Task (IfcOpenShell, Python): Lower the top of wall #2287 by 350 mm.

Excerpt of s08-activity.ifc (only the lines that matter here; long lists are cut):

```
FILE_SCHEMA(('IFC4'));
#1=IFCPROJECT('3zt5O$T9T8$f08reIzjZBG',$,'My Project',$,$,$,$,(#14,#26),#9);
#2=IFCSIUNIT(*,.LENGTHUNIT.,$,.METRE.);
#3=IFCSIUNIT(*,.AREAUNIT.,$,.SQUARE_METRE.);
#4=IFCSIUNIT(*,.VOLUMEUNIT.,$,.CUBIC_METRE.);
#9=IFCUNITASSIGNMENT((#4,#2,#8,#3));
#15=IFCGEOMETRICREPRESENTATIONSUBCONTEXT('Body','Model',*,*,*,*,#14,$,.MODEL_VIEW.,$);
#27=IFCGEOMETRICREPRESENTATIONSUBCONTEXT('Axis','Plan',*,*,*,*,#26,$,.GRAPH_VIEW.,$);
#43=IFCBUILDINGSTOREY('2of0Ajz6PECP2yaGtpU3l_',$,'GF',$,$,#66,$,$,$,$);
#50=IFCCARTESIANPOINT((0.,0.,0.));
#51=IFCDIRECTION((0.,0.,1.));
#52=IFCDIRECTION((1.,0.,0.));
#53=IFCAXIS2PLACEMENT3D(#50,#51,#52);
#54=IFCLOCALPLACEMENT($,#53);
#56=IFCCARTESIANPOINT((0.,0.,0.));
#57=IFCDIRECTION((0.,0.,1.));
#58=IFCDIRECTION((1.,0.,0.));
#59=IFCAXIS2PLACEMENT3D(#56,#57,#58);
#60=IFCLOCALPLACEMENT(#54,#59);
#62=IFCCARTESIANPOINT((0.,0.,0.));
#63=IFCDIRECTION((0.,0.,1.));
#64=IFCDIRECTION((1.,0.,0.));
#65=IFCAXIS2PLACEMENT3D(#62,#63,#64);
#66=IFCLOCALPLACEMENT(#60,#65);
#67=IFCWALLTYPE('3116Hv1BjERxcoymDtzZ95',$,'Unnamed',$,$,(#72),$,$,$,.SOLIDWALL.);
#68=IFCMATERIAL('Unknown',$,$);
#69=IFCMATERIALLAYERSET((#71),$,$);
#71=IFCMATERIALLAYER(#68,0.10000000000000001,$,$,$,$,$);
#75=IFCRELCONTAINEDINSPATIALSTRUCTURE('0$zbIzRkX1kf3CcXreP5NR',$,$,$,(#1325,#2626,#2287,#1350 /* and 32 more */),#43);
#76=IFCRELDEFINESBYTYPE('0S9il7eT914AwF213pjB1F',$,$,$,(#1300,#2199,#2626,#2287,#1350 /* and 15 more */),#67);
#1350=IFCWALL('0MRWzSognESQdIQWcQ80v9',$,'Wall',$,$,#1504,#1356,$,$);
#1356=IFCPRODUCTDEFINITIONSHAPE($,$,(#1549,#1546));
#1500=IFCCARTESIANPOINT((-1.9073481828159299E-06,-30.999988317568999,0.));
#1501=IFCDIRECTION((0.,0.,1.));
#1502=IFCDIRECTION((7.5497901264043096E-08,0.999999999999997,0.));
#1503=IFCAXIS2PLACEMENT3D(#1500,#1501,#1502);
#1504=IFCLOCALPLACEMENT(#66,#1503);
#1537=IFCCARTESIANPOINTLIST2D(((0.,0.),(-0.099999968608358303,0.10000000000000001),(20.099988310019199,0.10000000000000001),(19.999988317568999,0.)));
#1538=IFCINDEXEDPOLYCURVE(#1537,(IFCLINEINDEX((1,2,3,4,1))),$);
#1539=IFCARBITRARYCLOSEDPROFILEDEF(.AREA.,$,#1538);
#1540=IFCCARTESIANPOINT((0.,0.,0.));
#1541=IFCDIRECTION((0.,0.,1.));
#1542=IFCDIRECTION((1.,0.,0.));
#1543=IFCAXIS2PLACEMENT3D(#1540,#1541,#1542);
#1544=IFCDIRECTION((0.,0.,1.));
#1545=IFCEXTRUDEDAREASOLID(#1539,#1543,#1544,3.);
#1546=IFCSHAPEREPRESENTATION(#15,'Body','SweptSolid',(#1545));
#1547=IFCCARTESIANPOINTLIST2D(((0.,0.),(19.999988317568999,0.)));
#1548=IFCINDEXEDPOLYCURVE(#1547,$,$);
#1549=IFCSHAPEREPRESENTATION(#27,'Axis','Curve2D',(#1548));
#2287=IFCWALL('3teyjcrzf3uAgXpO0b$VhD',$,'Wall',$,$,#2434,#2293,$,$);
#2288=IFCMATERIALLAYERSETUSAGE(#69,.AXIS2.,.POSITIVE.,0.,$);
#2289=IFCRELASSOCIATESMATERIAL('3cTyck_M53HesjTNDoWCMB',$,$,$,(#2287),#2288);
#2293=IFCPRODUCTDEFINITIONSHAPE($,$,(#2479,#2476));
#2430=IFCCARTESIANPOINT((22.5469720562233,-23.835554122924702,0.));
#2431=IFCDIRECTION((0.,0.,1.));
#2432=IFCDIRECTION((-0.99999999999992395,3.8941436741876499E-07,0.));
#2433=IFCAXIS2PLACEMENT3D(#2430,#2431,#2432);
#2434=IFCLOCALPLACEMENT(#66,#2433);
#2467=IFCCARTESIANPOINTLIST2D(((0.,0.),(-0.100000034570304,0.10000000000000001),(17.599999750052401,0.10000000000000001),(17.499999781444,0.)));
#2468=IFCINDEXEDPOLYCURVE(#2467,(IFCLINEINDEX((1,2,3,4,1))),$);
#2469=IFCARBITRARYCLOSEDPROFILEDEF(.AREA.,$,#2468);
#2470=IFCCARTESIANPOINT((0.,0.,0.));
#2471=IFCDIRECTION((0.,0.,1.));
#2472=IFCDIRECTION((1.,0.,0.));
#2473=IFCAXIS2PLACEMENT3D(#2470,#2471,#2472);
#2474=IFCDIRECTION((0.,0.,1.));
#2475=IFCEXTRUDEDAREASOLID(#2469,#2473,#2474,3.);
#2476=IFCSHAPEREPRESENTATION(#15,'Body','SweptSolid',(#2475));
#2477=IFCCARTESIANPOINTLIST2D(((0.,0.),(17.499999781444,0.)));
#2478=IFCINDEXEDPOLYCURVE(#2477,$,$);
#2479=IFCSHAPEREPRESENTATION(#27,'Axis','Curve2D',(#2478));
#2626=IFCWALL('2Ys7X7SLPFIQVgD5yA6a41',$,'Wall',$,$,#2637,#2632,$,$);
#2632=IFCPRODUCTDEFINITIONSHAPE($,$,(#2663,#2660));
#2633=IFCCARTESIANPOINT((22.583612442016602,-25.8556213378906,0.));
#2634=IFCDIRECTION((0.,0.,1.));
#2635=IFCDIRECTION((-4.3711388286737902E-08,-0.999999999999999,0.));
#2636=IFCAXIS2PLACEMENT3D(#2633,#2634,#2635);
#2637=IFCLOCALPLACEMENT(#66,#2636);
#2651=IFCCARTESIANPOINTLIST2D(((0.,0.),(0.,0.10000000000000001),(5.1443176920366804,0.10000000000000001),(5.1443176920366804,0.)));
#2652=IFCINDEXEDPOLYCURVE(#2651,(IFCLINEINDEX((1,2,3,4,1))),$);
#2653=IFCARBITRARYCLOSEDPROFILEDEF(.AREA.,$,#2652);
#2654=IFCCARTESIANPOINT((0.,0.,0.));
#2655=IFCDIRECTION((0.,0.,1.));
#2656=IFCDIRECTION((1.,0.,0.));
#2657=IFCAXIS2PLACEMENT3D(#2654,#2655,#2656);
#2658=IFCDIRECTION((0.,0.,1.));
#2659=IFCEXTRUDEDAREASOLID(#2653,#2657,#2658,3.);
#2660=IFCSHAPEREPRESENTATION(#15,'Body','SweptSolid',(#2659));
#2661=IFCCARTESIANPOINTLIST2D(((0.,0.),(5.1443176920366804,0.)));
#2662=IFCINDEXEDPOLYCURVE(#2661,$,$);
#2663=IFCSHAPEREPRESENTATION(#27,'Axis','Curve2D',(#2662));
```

```python
import ifcopenshell
import ifcopenshell.geom
import ifcopenshell.util.representation
import ifcopenshell.util.shape

model = ifcopenshell.open("s08-activity.ifc")
settings = ifcopenshell.geom.settings()


def volume(element):
    """Net volume in cubic metres, openings subtracted."""
    shape = ifcopenshell.geom.create_shape(settings, element)
    return ifcopenshell.util.shape.get_volume(shape.geometry)


wall = model.by_guid("3teyjcrzf3uAgXpO0b$VhD")
before = volume(wall)

body = ifcopenshell.util.representation.get_representation(wall, "Model", "Body")
solid = body.Items[0]
old_height = solid.Depth
solid.Depth -= 0.35
after = volume(wall)

print(f"height {old_height:g} -> {solid.Depth:g}, volume {before:.3f} -> {after:.3f} m3")

model.write("s08-activity_rev.ifc")
```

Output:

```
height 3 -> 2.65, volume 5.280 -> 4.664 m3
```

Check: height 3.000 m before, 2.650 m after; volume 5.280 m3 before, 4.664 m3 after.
